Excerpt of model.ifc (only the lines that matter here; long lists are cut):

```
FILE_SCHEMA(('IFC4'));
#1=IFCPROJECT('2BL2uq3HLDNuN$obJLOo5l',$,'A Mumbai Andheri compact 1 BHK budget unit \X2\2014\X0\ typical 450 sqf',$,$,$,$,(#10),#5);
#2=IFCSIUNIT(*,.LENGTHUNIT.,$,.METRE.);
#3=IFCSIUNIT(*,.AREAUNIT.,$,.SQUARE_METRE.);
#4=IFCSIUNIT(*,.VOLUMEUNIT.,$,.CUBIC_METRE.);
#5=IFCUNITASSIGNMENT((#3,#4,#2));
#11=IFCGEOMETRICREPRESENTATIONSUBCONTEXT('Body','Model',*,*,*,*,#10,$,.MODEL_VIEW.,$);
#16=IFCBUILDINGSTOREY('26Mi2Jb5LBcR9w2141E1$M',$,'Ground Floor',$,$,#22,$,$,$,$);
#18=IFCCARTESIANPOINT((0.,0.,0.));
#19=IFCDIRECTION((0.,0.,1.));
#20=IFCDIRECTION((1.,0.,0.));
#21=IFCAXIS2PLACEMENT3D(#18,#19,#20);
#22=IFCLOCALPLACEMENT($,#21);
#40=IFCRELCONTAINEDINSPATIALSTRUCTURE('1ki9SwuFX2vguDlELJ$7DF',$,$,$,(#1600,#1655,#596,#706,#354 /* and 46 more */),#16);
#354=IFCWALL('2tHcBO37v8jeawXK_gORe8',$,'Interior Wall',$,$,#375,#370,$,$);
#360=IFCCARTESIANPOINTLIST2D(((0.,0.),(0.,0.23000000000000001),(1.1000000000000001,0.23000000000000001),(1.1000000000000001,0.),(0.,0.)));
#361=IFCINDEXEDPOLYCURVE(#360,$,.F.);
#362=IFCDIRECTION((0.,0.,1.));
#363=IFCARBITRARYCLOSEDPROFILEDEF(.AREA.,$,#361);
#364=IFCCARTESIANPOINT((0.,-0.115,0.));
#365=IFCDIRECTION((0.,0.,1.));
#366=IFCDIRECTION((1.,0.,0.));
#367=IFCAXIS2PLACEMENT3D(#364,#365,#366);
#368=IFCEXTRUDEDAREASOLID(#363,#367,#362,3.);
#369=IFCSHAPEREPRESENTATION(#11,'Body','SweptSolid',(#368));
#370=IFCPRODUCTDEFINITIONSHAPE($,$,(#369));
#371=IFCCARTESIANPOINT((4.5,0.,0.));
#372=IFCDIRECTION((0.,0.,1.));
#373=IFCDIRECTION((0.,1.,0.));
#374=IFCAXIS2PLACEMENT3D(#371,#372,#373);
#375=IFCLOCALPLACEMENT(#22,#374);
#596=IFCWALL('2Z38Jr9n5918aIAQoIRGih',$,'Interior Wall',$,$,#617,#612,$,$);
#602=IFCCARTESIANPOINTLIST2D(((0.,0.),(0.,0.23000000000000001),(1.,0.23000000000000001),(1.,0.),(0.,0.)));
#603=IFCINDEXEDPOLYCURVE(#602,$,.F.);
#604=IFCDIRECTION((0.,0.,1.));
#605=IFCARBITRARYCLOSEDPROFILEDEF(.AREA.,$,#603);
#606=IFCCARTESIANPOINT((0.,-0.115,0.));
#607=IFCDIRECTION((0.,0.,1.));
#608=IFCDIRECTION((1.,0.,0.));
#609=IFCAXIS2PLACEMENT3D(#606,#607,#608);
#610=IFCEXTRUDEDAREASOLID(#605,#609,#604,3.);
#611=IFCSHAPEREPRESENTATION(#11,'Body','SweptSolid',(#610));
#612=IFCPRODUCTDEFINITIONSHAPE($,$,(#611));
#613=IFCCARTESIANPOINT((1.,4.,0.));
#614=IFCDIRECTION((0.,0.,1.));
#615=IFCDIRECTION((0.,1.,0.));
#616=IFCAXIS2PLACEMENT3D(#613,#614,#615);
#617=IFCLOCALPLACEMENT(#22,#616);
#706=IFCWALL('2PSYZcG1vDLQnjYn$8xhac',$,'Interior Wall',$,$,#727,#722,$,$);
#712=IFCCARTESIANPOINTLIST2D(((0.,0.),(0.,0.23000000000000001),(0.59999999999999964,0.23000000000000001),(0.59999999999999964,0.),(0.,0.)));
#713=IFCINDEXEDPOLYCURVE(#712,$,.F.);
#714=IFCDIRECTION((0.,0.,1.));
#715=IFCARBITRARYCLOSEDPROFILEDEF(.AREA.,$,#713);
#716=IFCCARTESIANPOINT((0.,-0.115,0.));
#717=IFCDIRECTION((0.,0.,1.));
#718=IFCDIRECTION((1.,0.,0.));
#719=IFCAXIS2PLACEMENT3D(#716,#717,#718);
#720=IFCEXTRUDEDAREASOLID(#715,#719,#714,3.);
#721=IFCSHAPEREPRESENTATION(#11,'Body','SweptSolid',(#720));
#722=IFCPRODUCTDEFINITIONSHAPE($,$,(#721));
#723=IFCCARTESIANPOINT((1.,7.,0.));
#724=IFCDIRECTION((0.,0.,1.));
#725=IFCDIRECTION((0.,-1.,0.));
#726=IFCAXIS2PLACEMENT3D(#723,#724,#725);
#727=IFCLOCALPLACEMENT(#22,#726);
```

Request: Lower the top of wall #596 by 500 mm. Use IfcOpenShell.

```python
import ifcopenshell
import ifcopenshell.geom
import ifcopenshell.util.representation
import ifcopenshell.util.shape
import ifcopenshell.util.unit

model = ifcopenshell.open("model.ifc")
unit_scale = ifcopenshell.util.unit.calculate_unit_scale(model)
settings = ifcopenshell.geom.settings()


def volume(element):
    """Net volume in cubic metres, openings subtracted."""
    shape = ifcopenshell.geom.create_shape(settings, element)
    return ifcopenshell.util.shape.get_volume(shape.geometry)


wall = model.by_guid("2Z38Jr9n5918aIAQoIRGih")
before = volume(wall)

body = ifcopenshell.util.representation.get_representation(wall, "Model", "Body")
solid = body.Items[0]
old_height = solid.Depth
solid.Depth -= 0.5 / unit_scale
after = volume(wall)

print(f"height {old_height:g} -> {solid.Depth:g}, volume {before:.3f} -> {after:.3f} m3")

model.write("model_rev.ifc")
```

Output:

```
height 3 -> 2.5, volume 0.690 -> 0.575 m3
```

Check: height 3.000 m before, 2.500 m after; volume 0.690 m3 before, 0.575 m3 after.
